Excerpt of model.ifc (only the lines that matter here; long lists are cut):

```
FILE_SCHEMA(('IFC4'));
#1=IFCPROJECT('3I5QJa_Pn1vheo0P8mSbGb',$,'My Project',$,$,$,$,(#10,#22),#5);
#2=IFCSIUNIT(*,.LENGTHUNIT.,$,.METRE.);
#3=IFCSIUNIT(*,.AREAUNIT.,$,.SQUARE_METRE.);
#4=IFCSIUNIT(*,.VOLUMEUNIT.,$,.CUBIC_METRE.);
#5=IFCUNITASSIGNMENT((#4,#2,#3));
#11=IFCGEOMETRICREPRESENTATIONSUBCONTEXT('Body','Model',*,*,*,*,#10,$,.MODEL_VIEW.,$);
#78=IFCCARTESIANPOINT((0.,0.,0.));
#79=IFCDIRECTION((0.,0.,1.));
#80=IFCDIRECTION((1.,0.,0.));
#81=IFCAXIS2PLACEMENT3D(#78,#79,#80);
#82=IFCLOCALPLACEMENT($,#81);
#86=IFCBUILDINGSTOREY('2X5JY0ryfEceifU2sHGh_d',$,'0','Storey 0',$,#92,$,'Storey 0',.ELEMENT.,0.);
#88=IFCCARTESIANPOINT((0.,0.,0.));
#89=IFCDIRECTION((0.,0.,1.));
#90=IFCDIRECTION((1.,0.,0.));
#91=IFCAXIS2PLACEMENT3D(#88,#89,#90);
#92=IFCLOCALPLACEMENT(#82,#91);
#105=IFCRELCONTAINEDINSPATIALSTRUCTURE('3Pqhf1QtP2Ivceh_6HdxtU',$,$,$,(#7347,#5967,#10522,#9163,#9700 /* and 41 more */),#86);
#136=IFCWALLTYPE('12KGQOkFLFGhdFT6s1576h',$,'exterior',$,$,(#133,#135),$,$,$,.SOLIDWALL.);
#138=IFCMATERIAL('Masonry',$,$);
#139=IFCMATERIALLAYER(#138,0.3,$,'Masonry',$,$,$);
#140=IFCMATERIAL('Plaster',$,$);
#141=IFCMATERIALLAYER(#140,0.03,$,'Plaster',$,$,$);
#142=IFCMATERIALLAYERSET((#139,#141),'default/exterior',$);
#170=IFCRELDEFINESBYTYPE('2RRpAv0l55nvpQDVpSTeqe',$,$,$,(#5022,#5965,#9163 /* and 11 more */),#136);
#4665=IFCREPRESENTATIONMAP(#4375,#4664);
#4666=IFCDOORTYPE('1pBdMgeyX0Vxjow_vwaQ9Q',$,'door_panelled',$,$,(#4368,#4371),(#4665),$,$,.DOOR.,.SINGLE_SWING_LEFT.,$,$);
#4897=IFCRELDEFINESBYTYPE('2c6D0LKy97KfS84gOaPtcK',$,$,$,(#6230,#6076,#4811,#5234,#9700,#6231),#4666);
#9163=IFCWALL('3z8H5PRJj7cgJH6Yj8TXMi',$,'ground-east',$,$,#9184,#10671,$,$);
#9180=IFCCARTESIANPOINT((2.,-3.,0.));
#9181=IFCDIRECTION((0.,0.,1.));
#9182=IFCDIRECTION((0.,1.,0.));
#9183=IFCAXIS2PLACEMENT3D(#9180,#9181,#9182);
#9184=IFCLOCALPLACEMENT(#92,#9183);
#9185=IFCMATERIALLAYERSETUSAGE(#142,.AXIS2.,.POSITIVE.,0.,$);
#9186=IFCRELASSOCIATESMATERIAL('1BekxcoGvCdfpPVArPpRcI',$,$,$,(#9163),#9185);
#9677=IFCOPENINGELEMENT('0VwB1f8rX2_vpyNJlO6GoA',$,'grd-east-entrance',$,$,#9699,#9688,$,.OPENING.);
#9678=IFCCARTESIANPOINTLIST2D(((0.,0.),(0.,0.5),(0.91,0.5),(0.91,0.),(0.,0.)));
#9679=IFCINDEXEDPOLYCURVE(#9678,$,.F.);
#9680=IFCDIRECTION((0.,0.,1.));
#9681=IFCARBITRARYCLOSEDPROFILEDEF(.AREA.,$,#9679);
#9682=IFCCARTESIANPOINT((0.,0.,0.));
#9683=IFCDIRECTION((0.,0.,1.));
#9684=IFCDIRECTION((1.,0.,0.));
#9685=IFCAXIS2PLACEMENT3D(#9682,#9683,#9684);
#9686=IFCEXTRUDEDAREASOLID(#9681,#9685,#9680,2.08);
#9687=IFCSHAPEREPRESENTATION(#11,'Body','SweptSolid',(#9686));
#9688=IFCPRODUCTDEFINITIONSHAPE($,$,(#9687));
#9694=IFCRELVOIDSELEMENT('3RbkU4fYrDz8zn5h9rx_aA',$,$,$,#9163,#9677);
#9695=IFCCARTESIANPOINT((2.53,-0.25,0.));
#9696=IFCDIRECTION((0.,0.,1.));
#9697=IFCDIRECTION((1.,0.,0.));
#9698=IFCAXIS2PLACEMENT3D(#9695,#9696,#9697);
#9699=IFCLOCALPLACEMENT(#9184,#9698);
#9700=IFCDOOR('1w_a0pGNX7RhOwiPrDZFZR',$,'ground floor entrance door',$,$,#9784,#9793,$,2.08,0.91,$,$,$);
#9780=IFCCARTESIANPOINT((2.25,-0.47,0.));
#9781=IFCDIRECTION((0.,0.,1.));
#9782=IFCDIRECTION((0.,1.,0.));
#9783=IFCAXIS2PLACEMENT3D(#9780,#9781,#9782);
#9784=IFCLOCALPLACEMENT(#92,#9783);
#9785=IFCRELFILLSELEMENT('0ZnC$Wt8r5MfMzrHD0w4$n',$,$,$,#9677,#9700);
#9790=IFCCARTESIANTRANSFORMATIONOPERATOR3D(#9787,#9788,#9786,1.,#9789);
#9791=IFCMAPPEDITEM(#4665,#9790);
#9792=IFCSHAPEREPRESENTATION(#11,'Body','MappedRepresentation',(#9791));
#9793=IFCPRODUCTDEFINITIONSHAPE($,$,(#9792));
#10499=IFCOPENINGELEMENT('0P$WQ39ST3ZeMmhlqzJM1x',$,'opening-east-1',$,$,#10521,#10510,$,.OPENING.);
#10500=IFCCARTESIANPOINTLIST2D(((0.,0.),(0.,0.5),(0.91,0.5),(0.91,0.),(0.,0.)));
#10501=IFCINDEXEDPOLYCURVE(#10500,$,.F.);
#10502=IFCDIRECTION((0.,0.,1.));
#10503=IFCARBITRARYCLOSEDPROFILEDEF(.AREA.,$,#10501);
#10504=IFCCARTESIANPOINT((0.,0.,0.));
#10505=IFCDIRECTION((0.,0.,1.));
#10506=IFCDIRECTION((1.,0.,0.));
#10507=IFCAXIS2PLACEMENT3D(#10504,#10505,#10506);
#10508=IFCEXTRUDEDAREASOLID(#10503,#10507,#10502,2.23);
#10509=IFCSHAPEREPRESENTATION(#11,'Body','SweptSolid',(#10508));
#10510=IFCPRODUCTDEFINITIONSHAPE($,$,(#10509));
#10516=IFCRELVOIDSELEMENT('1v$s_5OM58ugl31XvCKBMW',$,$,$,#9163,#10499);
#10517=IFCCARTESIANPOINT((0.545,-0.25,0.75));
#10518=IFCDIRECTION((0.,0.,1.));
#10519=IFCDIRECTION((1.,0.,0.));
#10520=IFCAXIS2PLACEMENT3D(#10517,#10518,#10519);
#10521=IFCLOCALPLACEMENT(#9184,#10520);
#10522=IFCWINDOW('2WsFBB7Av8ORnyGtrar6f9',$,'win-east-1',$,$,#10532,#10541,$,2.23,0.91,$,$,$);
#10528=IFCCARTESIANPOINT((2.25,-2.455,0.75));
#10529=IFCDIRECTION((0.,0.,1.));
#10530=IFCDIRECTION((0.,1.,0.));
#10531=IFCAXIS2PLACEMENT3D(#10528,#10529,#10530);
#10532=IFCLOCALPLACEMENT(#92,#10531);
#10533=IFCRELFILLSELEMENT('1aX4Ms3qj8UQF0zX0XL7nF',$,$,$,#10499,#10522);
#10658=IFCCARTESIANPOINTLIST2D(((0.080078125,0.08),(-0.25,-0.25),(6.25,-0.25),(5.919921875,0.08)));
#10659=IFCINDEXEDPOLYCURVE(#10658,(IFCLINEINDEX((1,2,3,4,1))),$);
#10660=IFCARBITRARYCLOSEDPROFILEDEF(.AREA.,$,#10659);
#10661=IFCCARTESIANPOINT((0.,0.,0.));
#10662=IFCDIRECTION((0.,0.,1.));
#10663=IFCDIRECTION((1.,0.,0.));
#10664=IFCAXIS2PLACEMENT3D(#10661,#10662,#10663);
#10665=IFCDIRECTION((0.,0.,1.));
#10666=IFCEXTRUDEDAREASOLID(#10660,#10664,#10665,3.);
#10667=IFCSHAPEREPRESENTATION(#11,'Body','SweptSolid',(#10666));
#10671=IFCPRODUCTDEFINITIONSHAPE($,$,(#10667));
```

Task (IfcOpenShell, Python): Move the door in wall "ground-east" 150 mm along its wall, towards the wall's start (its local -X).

```python
import ifcopenshell
import ifcopenshell.api.geometry
import ifcopenshell.util.placement
import ifcopenshell.util.unit

model = ifcopenshell.open("model.ifc")
unit_scale = ifcopenshell.util.unit.calculate_unit_scale(model)

door = model.by_guid("1w_a0pGNX7RhOwiPrDZFZR")
opening = door.FillsVoids[0].RelatingOpeningElement
wall = opening.VoidsElements[0].RelatingBuildingElement

wall_matrix = ifcopenshell.util.placement.get_local_placement(wall.ObjectPlacement)
shift = wall_matrix[:3, 0] * -0.15 / unit_scale
before = ifcopenshell.util.placement.get_local_placement(door.ObjectPlacement)[:3, 3].copy()

# The door is not placed relative to its opening, so move both.
for product in (opening, door):
    matrix = ifcopenshell.util.placement.get_local_placement(product.ObjectPlacement)
    matrix[:3, 3] += shift
    ifcopenshell.api.geometry.edit_object_placement(model, product=product, matrix=matrix, is_si=False)

after = ifcopenshell.util.placement.get_local_placement(door.ObjectPlacement)[:3, 3]
print("door moved by", (after - before).round(3) + 0.0)

model.write("model_rev.ifc")
```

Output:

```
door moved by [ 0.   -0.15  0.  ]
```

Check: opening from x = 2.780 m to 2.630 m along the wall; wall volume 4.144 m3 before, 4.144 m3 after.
